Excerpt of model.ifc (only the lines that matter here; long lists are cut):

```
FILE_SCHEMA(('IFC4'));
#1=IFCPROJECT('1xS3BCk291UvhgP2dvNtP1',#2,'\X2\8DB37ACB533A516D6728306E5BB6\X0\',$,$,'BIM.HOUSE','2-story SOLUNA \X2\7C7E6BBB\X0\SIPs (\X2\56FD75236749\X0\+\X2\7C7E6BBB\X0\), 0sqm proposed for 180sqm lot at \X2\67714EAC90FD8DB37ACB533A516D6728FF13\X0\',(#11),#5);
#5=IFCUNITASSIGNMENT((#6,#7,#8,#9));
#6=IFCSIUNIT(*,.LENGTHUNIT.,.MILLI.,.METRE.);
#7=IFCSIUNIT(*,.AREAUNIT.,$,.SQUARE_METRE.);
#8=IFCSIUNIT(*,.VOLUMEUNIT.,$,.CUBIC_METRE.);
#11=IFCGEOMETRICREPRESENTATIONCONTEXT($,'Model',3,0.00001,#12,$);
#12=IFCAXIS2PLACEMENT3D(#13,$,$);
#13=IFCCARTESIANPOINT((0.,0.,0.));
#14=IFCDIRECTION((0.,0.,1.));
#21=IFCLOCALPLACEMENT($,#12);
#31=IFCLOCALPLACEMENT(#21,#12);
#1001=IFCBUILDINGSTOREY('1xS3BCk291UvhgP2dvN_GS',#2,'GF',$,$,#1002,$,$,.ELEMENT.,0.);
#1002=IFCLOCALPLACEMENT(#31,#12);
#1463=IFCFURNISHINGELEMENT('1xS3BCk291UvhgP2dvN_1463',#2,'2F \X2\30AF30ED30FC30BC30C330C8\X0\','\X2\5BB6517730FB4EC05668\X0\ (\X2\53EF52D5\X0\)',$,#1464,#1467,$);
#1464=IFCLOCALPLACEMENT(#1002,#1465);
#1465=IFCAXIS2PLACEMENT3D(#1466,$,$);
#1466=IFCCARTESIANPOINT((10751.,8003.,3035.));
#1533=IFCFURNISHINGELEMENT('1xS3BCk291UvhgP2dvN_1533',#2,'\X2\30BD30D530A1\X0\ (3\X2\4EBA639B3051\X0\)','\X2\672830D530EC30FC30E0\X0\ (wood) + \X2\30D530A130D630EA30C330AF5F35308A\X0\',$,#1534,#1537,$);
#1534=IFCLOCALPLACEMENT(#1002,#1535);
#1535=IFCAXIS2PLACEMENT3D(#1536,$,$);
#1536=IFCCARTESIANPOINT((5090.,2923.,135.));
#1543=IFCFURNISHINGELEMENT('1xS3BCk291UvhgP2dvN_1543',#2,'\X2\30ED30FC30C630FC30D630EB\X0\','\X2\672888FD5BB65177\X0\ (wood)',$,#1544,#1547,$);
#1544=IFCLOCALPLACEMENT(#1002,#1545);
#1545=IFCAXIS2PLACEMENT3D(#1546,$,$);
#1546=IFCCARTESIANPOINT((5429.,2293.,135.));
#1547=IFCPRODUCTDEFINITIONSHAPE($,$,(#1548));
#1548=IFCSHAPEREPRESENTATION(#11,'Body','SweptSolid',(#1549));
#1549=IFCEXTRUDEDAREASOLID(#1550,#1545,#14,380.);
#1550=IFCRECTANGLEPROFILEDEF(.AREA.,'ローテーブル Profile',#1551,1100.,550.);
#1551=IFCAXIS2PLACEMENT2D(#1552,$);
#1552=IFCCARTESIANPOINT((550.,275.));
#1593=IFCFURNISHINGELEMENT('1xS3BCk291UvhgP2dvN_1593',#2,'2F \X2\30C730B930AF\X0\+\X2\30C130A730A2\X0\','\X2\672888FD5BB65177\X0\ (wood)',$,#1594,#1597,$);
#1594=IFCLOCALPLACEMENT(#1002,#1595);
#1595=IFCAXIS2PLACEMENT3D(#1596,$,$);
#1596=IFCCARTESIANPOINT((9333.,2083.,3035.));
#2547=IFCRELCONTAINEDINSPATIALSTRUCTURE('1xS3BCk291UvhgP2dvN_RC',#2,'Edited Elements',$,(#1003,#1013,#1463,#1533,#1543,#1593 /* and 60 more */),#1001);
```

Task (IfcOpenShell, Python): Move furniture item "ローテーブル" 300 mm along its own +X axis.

```python
import ifcopenshell
import ifcopenshell.api.geometry
import ifcopenshell.util.placement
import ifcopenshell.util.unit

model = ifcopenshell.open("model.ifc")
unit_scale = ifcopenshell.util.unit.calculate_unit_scale(model)

item = model.by_guid("1xS3BCk291UvhgP2dvN_1543")
matrix = ifcopenshell.util.placement.get_local_placement(item.ObjectPlacement)
matrix[:3, 3] += matrix[:3, 0] * 0.3 / unit_scale
ifcopenshell.api.geometry.edit_object_placement(model, product=item, matrix=matrix, is_si=False)

print(ifcopenshell.util.placement.get_local_placement(item.ObjectPlacement).round(3) + 0.0)

model.write("model_edited.ifc")
```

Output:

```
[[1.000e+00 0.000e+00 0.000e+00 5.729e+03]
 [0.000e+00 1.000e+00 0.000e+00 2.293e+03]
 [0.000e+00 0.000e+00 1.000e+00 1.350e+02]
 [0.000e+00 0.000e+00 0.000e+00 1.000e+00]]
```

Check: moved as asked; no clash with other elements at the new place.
